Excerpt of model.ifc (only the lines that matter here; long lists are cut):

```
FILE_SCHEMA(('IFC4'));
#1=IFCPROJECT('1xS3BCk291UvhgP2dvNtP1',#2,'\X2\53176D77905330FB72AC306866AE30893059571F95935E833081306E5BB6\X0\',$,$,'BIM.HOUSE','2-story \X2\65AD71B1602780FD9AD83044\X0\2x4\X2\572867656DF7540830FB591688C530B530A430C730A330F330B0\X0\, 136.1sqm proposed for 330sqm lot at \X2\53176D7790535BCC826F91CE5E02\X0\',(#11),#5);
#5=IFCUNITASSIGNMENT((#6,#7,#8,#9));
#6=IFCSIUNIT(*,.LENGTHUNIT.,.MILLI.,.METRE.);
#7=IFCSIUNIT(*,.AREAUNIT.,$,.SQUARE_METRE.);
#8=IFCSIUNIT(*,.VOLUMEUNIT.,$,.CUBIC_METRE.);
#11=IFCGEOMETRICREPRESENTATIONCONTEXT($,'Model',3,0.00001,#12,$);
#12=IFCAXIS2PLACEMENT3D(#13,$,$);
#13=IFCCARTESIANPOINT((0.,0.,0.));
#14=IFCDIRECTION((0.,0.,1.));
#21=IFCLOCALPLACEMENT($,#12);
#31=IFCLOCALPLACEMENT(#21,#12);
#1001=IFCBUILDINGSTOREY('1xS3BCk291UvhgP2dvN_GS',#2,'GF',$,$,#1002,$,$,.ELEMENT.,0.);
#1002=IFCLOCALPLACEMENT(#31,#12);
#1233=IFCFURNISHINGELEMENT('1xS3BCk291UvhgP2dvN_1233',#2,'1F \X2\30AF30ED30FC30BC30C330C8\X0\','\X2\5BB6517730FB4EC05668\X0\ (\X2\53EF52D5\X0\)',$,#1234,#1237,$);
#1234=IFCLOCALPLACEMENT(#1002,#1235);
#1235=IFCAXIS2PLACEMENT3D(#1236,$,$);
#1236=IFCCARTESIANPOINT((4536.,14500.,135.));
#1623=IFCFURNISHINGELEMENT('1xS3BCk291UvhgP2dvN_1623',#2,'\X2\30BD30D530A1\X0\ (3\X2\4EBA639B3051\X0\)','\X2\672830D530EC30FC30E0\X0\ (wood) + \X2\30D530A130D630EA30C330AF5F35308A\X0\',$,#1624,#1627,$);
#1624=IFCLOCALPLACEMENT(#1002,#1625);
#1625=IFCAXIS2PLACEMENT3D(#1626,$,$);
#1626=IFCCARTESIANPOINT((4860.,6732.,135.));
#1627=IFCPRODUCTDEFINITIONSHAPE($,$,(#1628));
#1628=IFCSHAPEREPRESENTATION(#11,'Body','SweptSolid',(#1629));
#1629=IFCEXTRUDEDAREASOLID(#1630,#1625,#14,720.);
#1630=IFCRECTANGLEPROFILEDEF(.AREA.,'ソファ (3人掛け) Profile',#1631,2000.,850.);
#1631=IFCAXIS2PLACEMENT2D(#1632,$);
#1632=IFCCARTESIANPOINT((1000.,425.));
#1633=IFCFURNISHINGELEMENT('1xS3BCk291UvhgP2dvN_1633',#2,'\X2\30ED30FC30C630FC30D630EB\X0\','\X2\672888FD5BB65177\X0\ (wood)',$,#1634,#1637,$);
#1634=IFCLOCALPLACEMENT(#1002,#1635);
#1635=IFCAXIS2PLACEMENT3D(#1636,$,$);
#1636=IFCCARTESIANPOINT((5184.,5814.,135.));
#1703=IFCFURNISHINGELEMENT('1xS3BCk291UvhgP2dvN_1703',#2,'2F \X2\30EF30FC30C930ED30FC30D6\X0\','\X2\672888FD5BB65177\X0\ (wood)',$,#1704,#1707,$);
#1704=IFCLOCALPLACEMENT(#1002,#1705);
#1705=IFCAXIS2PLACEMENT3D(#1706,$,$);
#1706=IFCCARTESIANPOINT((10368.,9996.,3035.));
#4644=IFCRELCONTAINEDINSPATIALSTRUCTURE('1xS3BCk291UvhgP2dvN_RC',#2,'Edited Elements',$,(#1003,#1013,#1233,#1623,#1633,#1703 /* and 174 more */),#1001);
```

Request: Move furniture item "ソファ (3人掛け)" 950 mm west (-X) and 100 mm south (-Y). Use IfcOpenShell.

```python
import ifcopenshell
import ifcopenshell.api.geometry
import ifcopenshell.util.placement
import ifcopenshell.util.unit

model = ifcopenshell.open("model.ifc")
unit_scale = ifcopenshell.util.unit.calculate_unit_scale(model)

item = model.by_guid("1xS3BCk291UvhgP2dvN_1623")
matrix = ifcopenshell.util.placement.get_local_placement(item.ObjectPlacement)
matrix[0, 3] -= 0.95 / unit_scale
matrix[1, 3] -= 0.1 / unit_scale
ifcopenshell.api.geometry.edit_object_placement(model, product=item, matrix=matrix, is_si=False)

print(ifcopenshell.util.placement.get_local_placement(item.ObjectPlacement).round(3) + 0.0)

model.write("model_rev.ifc")
```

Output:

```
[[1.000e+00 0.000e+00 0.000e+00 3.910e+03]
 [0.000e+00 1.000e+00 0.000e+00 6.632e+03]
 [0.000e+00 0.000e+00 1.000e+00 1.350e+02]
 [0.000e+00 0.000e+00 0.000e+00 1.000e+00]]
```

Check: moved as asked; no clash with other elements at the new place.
